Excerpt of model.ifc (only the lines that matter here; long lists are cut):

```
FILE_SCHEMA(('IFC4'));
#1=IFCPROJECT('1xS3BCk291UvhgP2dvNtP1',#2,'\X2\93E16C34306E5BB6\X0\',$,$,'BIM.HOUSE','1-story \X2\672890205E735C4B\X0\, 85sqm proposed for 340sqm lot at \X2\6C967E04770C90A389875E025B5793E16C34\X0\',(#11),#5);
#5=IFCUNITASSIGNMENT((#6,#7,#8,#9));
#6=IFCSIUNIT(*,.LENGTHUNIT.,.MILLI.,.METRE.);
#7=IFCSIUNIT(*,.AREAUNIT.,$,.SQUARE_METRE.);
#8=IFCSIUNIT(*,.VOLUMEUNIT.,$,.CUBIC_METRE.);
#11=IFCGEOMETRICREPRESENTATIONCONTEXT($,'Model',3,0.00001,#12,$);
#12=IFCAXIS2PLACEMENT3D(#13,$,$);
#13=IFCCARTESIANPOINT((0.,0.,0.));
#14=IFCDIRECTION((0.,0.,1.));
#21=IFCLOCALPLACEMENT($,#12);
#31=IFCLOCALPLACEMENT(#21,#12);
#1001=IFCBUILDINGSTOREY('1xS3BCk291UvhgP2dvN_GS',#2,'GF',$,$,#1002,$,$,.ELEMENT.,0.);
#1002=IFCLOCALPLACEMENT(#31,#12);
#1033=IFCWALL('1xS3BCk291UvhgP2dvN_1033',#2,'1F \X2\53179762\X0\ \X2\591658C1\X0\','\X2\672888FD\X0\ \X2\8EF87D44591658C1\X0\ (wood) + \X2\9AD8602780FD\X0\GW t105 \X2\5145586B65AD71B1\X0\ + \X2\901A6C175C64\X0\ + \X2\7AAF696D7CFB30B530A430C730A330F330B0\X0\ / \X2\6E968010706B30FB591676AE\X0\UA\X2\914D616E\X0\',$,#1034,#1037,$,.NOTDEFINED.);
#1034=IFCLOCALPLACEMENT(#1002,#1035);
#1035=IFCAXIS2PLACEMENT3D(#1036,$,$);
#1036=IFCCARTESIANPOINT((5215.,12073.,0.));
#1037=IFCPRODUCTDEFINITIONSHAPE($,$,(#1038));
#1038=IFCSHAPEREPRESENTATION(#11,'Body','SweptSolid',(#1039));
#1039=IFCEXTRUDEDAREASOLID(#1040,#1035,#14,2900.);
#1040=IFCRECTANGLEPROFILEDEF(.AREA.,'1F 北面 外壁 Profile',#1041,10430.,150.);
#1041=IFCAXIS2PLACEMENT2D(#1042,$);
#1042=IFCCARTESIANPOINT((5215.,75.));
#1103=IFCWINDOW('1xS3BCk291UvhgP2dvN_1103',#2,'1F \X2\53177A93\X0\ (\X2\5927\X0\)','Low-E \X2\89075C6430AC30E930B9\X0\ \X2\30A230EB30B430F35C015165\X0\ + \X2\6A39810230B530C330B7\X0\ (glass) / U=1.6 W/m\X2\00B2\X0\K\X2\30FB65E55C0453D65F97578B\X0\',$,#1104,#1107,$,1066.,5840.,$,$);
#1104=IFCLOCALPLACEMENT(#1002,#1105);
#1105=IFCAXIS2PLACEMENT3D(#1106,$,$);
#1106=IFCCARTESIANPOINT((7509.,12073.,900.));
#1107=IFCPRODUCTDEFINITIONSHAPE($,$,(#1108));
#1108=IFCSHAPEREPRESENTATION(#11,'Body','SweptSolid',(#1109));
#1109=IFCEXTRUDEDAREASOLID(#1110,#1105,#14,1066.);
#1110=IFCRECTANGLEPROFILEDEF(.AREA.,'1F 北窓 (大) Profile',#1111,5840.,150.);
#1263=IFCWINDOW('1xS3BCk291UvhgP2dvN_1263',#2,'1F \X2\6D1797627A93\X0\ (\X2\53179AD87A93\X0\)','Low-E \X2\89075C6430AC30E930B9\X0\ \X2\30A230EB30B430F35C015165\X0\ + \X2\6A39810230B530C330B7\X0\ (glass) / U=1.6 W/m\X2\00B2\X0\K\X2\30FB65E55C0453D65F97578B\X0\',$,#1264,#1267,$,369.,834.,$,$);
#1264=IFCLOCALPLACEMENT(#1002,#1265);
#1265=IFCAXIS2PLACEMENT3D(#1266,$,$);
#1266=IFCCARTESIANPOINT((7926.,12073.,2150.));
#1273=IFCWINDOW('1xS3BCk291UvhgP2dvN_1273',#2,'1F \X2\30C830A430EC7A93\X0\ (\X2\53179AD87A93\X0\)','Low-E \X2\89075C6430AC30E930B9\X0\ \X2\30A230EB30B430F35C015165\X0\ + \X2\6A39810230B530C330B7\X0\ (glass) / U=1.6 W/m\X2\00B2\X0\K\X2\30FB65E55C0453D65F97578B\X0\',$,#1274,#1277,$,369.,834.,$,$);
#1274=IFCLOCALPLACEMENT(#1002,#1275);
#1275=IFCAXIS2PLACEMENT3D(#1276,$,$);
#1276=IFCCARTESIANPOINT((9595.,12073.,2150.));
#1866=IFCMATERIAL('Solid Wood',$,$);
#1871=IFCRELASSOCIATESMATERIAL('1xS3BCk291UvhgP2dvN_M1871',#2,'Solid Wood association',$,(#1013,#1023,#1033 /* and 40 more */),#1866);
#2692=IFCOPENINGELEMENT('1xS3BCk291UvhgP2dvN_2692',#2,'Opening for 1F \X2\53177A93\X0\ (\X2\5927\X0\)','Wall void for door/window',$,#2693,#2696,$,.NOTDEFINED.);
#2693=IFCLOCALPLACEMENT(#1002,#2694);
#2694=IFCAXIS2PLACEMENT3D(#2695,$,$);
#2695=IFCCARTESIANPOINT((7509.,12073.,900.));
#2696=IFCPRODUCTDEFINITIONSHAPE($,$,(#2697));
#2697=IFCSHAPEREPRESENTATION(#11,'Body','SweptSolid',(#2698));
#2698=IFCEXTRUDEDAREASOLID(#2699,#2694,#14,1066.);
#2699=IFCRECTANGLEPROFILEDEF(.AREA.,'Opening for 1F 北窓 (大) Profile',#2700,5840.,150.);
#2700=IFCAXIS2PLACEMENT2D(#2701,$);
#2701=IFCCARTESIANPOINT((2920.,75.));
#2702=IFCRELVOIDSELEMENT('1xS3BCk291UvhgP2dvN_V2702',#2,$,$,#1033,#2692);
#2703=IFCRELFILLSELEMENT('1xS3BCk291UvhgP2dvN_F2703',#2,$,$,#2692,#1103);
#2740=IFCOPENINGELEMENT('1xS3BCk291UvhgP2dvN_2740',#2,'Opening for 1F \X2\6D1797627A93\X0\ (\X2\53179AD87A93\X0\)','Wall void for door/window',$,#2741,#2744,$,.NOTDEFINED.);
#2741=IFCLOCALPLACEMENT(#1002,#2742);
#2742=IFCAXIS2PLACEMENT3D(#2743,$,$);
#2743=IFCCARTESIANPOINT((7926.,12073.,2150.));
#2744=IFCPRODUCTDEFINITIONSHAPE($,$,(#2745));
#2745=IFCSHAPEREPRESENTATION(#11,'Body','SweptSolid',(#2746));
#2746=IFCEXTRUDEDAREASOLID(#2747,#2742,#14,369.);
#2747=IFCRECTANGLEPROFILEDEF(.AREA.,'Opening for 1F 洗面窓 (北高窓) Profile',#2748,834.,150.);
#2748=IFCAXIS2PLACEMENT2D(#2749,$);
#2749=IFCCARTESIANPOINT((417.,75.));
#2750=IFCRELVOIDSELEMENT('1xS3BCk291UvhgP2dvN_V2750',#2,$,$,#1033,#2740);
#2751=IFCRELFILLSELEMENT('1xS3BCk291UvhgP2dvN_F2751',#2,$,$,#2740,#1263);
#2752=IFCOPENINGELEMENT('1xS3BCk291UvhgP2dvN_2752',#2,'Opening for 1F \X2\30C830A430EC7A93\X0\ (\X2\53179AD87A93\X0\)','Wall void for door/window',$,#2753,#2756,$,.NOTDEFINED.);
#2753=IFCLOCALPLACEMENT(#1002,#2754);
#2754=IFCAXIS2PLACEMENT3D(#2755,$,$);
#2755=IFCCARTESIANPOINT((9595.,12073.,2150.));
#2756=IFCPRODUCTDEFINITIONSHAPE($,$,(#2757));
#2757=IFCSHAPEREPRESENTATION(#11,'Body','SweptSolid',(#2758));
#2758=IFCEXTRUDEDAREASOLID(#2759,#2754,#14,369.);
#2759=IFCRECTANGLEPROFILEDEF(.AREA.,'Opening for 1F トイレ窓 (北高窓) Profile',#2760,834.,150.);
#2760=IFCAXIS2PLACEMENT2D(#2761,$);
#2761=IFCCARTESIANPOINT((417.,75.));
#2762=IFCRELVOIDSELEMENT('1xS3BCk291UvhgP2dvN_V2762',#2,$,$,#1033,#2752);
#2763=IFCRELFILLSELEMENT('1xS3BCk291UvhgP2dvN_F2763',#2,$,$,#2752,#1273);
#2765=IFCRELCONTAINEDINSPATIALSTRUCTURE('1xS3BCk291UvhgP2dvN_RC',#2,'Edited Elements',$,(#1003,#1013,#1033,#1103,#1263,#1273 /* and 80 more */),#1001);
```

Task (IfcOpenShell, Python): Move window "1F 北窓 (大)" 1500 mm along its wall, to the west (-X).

```python
import ifcopenshell
import ifcopenshell.api.geometry
import ifcopenshell.util.placement
import ifcopenshell.util.unit

model = ifcopenshell.open("model.ifc")
unit_scale = ifcopenshell.util.unit.calculate_unit_scale(model)

window = model.by_id(1103)
opening = window.FillsVoids[0].RelatingOpeningElement
wall = opening.VoidsElements[0].RelatingBuildingElement

wall_matrix = ifcopenshell.util.placement.get_local_placement(wall.ObjectPlacement)
shift = wall_matrix[:3, 0] * -1.5 / unit_scale
before = ifcopenshell.util.placement.get_local_placement(window.ObjectPlacement)[:3, 3].copy()

# The window is not placed relative to its opening, so move both.
for product in (opening, window):
    matrix = ifcopenshell.util.placement.get_local_placement(product.ObjectPlacement)
    matrix[:3, 3] += shift
    ifcopenshell.api.geometry.edit_object_placement(model, product=product, matrix=matrix, is_si=False)

after = ifcopenshell.util.placement.get_local_placement(window.ObjectPlacement)[:3, 3]
print("window moved by", (after - before).round(3) + 0.0)

model.write("model_v2.ifc")
```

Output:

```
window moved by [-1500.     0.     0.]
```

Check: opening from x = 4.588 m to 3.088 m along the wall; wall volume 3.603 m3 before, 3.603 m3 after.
